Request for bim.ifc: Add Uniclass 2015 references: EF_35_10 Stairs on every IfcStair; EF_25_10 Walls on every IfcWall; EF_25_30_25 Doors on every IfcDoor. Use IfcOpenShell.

First a look at what the model holds.

```python
import ifcopenshell

model = ifcopenshell.open("bim.ifc")
print(model.schema)
print("classifications:", [c.Name for c in model.by_type("IfcClassification")])
for ifc_class in ("IfcDoor", "IfcRoof", "IfcStair", "IfcWall", "IfcWindow"):
    print(ifc_class, len(model.by_type(ifc_class)))
```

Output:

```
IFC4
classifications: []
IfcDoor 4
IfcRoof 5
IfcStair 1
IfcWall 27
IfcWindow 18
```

```python
import ifcopenshell
import ifcopenshell.api.classification

model = ifcopenshell.open("bim.ifc")

system = ifcopenshell.api.classification.add_classification(model, classification="Uniclass 2015")

codes = {
    "IfcStair": ("EF_35_10", "Stairs"),
    "IfcWall": ("EF_25_10", "Walls"),
    "IfcDoor": ("EF_25_30_25", "Doors"),
}
for ifc_class, (code, name) in codes.items():
    products = model.by_type(ifc_class)
    ifcopenshell.api.classification.add_reference(
        model, products=products, classification=system, identification=code, name=name
    )
    print(code, len(products))

model.write("bim-out.ifc")
```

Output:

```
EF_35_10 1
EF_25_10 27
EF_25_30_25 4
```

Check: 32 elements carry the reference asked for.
